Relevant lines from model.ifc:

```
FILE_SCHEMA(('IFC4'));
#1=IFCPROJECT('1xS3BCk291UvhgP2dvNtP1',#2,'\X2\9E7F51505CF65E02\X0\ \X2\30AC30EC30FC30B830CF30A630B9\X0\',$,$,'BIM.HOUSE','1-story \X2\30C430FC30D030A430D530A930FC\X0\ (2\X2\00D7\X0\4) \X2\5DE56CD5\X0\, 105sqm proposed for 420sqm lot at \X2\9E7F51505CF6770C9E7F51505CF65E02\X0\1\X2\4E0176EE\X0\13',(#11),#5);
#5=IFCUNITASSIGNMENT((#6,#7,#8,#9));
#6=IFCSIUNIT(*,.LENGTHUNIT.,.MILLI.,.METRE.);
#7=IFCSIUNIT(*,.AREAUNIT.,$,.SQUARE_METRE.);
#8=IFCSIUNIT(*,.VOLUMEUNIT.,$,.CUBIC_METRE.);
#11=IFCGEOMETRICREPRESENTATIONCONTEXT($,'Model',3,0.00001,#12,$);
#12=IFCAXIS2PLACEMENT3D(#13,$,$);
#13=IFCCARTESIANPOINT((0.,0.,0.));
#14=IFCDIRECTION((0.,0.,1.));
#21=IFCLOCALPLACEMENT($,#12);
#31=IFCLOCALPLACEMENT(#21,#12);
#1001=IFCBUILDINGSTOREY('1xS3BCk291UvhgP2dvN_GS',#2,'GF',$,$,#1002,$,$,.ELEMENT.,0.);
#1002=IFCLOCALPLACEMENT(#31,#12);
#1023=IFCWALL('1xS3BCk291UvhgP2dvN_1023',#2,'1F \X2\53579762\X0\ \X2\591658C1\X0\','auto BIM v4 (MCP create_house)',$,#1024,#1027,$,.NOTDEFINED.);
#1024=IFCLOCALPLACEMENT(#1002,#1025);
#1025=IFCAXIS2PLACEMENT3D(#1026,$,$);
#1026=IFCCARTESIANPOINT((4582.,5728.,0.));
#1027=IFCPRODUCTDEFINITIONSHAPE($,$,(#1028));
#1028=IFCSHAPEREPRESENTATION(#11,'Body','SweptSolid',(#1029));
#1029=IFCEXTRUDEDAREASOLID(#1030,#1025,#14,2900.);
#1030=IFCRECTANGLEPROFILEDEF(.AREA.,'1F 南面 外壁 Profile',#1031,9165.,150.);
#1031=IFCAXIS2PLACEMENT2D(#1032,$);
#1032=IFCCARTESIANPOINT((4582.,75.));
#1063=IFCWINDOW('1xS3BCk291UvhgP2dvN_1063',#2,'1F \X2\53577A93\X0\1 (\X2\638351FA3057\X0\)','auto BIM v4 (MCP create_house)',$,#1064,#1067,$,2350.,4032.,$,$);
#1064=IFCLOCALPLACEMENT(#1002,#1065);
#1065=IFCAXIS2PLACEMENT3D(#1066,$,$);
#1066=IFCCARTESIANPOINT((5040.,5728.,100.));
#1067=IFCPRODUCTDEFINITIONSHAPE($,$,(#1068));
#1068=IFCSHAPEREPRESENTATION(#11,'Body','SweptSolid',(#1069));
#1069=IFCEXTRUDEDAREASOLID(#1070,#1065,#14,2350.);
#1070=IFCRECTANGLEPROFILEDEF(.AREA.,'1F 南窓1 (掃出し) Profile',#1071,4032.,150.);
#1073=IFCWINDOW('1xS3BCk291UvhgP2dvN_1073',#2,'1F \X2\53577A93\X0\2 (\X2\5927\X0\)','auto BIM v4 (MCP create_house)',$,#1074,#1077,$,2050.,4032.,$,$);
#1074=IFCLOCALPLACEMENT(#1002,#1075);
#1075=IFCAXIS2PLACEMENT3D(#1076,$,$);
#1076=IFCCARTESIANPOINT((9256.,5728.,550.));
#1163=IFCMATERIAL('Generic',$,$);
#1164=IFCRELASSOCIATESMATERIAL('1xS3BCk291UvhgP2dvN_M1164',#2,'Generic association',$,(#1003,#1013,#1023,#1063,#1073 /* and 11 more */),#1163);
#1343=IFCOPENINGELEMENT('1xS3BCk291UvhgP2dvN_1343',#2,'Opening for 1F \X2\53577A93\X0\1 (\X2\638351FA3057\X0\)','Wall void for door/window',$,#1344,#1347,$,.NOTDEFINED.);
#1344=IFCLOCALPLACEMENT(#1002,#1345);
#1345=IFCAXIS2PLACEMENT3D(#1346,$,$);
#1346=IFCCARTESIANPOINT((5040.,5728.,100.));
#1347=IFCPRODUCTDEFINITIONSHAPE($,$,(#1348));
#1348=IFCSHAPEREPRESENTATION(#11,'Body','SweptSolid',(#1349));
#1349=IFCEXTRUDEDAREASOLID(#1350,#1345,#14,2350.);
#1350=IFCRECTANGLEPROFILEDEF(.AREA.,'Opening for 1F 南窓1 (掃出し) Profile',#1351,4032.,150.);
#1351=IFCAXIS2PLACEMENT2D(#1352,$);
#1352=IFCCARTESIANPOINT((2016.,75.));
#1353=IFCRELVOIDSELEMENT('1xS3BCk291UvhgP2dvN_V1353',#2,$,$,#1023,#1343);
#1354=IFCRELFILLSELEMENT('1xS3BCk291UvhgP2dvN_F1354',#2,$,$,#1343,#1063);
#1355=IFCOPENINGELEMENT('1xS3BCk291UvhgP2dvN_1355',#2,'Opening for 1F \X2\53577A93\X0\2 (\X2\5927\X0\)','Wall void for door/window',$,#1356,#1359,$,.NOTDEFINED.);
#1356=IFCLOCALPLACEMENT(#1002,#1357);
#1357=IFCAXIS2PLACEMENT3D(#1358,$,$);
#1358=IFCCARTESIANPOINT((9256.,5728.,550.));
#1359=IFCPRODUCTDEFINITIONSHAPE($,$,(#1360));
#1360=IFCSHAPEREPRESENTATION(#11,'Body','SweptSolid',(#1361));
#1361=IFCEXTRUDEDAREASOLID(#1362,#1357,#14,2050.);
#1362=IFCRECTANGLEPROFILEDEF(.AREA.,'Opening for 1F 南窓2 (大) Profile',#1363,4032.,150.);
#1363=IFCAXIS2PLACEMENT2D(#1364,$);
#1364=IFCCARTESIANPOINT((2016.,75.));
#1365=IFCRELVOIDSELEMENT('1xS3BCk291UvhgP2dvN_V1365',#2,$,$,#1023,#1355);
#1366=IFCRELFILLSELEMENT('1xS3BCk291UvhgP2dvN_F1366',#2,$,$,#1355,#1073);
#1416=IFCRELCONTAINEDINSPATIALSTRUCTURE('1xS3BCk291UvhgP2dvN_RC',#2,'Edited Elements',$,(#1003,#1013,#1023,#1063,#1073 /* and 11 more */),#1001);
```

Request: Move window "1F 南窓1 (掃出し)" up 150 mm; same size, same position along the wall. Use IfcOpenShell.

```python
import numpy as np
import ifcopenshell
import ifcopenshell.api.geometry
import ifcopenshell.util.placement
import ifcopenshell.util.unit

model = ifcopenshell.open("model.ifc")
unit_scale = ifcopenshell.util.unit.calculate_unit_scale(model)

window = model.by_guid("1xS3BCk291UvhgP2dvN_1063")
opening = window.FillsVoids[0].RelatingOpeningElement
dz = 0.15 / unit_scale

shift = np.array([0.0, 0.0, dz])
# The window is not placed relative to its opening, so move both.
for product in (opening, window):
    matrix = ifcopenshell.util.placement.get_local_placement(product.ObjectPlacement)
    matrix[:3, 3] += shift
    ifcopenshell.api.geometry.edit_object_placement(model, product=product, matrix=matrix, is_si=False)

print(f"moved by {dz * unit_scale:+.3f} m")

model.write("model_v2.ifc")
```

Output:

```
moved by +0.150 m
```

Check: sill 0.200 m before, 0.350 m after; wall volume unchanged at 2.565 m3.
